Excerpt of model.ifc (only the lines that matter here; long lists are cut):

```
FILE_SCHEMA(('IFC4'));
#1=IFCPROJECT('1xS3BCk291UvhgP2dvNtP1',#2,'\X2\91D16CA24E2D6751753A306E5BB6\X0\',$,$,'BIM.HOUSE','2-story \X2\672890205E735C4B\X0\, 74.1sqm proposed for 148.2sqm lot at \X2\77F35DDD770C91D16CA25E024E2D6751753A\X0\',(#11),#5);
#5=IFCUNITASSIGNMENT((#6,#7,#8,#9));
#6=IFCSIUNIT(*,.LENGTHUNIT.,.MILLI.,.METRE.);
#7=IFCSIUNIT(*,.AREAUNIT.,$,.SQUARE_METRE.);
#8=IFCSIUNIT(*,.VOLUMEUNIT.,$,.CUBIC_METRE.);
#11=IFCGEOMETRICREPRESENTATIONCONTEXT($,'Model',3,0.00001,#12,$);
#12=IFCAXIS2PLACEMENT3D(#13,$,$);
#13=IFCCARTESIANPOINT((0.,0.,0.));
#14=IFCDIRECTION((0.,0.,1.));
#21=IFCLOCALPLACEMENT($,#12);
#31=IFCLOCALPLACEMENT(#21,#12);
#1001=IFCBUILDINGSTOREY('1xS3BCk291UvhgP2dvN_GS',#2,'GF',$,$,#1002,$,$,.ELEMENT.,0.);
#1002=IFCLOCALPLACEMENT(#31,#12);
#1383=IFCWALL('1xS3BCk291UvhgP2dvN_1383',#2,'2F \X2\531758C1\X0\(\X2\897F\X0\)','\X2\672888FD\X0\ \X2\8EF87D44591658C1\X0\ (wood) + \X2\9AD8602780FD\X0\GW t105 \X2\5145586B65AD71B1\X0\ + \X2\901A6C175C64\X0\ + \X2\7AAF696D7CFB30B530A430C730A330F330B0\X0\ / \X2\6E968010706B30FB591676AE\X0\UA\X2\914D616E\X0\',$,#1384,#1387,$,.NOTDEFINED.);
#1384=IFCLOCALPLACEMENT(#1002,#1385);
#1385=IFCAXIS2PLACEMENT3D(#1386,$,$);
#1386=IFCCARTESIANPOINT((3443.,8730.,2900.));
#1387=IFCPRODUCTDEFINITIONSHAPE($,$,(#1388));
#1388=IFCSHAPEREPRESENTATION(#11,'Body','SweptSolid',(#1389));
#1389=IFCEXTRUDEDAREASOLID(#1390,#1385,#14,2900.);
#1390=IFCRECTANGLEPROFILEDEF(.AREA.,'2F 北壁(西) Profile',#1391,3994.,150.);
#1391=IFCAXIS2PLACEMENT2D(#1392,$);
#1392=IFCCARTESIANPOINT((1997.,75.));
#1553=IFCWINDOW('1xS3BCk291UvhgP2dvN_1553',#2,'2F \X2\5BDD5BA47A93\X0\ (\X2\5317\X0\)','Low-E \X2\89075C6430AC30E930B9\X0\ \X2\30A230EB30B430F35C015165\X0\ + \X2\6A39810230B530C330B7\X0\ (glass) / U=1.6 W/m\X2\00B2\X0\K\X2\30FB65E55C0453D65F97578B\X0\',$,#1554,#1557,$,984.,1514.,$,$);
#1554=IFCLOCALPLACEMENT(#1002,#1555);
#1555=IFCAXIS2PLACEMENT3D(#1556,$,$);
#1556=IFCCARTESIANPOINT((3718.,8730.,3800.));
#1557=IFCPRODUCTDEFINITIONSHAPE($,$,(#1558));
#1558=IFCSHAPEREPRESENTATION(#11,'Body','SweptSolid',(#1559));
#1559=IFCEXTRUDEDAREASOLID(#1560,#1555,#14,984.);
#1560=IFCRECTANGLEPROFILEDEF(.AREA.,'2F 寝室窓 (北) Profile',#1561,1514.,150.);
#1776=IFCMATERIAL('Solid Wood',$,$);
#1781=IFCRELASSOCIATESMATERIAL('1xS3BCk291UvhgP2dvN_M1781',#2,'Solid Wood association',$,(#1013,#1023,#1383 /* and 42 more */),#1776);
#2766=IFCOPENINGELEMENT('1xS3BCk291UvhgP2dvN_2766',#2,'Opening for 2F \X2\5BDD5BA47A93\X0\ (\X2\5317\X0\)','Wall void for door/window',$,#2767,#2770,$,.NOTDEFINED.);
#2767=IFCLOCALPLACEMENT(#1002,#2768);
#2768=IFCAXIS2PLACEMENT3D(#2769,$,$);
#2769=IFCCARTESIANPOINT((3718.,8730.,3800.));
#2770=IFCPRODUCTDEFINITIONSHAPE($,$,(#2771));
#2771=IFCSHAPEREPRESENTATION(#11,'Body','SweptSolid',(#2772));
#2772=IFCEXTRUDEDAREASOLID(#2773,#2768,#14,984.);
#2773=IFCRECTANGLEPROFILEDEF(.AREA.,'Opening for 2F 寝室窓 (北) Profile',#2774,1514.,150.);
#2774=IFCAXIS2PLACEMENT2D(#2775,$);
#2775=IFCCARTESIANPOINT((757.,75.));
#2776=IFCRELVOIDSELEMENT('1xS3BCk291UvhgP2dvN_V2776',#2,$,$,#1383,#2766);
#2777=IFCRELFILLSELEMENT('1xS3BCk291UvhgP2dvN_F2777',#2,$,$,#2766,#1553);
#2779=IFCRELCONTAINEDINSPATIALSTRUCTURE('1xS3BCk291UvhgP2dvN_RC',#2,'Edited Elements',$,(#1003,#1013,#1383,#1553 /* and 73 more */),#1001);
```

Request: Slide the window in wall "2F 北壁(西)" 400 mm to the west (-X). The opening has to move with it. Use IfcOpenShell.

```python
import ifcopenshell
import ifcopenshell.api.geometry
import ifcopenshell.util.placement

model = ifcopenshell.open("model.ifc")

window = model.by_guid("1xS3BCk291UvhgP2dvN_1553")
opening = window.FillsVoids[0].RelatingOpeningElement
wall = opening.VoidsElements[0].RelatingBuildingElement

wall_matrix = ifcopenshell.util.placement.get_local_placement(wall.ObjectPlacement)
shift = wall_matrix[:3, 0] * -400.0
before = ifcopenshell.util.placement.get_local_placement(window.ObjectPlacement)[:3, 3].copy()

# The window is not placed relative to its opening, so move both.
for product in (opening, window):
    matrix = ifcopenshell.util.placement.get_local_placement(product.ObjectPlacement)
    matrix[:3, 3] += shift
    ifcopenshell.api.geometry.edit_object_placement(model, product=product, matrix=matrix, is_si=False)

after = ifcopenshell.util.placement.get_local_placement(window.ObjectPlacement)[:3, 3]
print("window moved by", (after - before).round(3) + 0.0)

model.write("model_rev.ifc")
```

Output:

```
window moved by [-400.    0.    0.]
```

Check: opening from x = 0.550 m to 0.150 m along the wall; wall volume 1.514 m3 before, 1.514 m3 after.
